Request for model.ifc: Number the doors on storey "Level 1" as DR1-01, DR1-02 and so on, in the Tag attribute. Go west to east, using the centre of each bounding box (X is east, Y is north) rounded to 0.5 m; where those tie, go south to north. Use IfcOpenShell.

First a look at what the model holds.

```python
import ifcopenshell
import ifcopenshell.util.element
import ifcopenshell.util.placement

model = ifcopenshell.open("model.ifc")
print(model.schema)
storey = next(s for s in model.by_type("IfcBuildingStorey") if s.Name == "Level 1")
doors = [e for e in ifcopenshell.util.element.get_decomposition(storey) if e.is_a("IfcDoor")]
for e in sorted(doors, key=lambda e: e.id()):
    origin = ifcopenshell.util.placement.get_local_placement(e.ObjectPlacement)[:3, 3]
    print(e.id(), e.Tag, e.Name, origin.round(2) + 0.0, sep=" | ")
```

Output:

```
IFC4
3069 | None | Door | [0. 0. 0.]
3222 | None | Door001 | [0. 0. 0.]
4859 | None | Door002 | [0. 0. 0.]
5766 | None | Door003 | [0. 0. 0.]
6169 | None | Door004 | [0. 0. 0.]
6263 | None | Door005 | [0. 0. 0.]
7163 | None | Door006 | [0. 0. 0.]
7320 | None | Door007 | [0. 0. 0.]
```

```python
import ifcopenshell
import ifcopenshell.geom
import ifcopenshell.util.element
import ifcopenshell.util.shape

model = ifcopenshell.open("model.ifc")
settings = ifcopenshell.geom.settings()
settings.set("use-world-coords", True)


def centre(element):
    shape = ifcopenshell.geom.create_shape(settings, element)
    return ifcopenshell.util.shape.get_bbox_centroid(shape.geometry)


storey = next(s for s in model.by_type("IfcBuildingStorey") if s.Name == "Level 1")
doors = [e for e in ifcopenshell.util.element.get_decomposition(storey) if e.is_a("IfcDoor")]

# Insertion points can sit at a corner or the storey origin, so sort by the geometry (in metres).
centres = {e: centre(e) for e in doors}
doors.sort(key=lambda e: (round(centres[e][0] / 0.5), centres[e][1]))

for i, e in enumerate(doors, start=1):
    number = f"DR1-{i:02d}"
    e.Tag = number
    print(e.id(), number)

model.write("model_v2.ifc")
```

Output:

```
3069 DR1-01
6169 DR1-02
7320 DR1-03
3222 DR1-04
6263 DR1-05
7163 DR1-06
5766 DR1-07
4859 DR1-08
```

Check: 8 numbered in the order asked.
